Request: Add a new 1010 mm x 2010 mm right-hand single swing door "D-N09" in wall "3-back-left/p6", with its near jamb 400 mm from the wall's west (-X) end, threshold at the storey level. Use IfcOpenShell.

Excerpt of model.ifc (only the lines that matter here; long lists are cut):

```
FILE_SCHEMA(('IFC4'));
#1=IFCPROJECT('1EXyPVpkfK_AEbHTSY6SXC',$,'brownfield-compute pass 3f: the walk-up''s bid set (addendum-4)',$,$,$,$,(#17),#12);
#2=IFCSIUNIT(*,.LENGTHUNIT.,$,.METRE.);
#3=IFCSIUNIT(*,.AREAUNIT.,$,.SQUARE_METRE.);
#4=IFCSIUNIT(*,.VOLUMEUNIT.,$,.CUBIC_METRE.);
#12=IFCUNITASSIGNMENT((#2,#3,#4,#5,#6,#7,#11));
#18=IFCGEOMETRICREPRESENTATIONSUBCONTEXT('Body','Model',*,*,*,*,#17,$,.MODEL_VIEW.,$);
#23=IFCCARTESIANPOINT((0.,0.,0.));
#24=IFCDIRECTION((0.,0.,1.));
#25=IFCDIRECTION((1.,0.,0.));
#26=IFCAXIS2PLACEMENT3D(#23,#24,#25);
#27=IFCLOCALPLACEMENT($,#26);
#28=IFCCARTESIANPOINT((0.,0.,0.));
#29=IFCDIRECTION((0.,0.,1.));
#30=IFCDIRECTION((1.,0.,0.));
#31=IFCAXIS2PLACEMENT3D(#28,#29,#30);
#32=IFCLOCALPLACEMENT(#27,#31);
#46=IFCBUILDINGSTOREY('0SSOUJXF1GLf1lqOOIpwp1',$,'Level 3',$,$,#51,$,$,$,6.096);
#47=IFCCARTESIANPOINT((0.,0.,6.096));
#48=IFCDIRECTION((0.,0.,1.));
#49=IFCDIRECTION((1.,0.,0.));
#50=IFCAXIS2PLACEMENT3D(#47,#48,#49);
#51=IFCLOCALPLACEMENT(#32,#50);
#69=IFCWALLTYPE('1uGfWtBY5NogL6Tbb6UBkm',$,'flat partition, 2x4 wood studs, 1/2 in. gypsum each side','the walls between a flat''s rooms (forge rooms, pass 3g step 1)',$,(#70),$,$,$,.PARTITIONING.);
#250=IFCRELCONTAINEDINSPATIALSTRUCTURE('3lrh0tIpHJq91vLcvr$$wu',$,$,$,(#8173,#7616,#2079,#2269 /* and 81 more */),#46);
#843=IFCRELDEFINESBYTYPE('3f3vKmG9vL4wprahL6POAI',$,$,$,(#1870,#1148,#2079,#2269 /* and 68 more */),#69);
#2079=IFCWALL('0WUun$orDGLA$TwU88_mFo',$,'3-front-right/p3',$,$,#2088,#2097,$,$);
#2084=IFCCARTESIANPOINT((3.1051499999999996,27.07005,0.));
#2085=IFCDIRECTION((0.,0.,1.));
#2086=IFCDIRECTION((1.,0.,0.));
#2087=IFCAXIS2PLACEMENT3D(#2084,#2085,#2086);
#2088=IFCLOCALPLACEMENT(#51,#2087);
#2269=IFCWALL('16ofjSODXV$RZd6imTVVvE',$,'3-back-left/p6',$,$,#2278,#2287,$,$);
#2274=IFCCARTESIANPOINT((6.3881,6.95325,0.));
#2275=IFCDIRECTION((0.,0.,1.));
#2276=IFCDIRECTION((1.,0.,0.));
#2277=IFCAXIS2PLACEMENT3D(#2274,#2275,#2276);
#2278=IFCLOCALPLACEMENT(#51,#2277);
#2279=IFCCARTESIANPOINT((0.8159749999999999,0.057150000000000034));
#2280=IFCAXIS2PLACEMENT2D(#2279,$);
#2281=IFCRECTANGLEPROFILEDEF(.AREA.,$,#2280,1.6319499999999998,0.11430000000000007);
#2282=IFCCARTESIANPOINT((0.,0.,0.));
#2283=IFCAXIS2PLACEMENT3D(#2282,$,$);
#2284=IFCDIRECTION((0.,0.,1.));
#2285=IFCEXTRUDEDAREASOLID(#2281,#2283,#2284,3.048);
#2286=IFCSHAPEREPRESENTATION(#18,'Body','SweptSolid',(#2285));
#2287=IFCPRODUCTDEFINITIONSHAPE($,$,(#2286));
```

```python
import numpy as np
import ifcopenshell
import ifcopenshell.api.feature
import ifcopenshell.api.geometry
import ifcopenshell.api.root
import ifcopenshell.api.spatial
import ifcopenshell.geom
import ifcopenshell.util.element
import ifcopenshell.util.placement
import ifcopenshell.util.representation
import ifcopenshell.util.shape
import ifcopenshell.util.unit

model = ifcopenshell.open("model.ifc")
unit_scale = ifcopenshell.util.unit.calculate_unit_scale(model)
settings = ifcopenshell.geom.settings()


def volume(element):
    """Net volume in cubic metres, openings subtracted."""
    shape = ifcopenshell.geom.create_shape(settings, element)
    return ifcopenshell.util.shape.get_volume(shape.geometry)


wall = model.by_id(2269)
storey = ifcopenshell.util.element.get_container(wall, ifc_class="IfcBuildingStorey")
context = ifcopenshell.util.representation.get_context(model, "Model", "Body", "MODEL_VIEW")
before = volume(wall)

width, height, from_end, sill = 1.01, 2.01, 0.4, 0.0  # metres

# The wall runs along its own X axis, and the end named is its -X end.
wall_shape = ifcopenshell.geom.create_shape(settings, wall)
x, y, z = ifcopenshell.util.shape.get_vertices(wall_shape.geometry).T
start = x.min() + from_end
face, thickness = float(y.min()), float(y.max() - y.min())
wall_matrix = ifcopenshell.util.placement.get_local_placement(wall.ObjectPlacement)
level = ifcopenshell.util.placement.get_local_placement(storey.ObjectPlacement)[2, 3]


def in_wall(x, y):
    """Placement at x, y metres in the wall's axes, at sill height."""
    matrix = wall_matrix.copy()
    matrix[:, 3] = wall_matrix @ np.array([x / unit_scale, y / unit_scale, 0.0, 1.0])
    matrix[2, 3] = level + sill / unit_scale
    return matrix


# Opening: a box that overshoots both wall faces by 50 mm.
opening = ifcopenshell.api.root.create_entity(model, ifc_class="IfcOpeningElement", predefined_type="OPENING")
box = ifcopenshell.api.geometry.add_wall_representation(
    model, context=context, length=width, height=height, thickness=thickness + 0.1
)
ifcopenshell.api.geometry.assign_representation(model, product=opening, representation=box)
ifcopenshell.api.geometry.edit_object_placement(model, product=opening, matrix=in_wall(start, face - 0.05), is_si=False)
ifcopenshell.api.feature.add_feature(model, feature=opening, element=wall)

door = ifcopenshell.api.root.create_entity(model, ifc_class="IfcDoor", name="D-N09", predefined_type="DOOR")
door.OverallWidth, door.OverallHeight = width / unit_scale, height / unit_scale
door.OperationType = "SINGLE_SWING_RIGHT"
body = ifcopenshell.api.geometry.add_door_representation(
    model,
    context=context,
    overall_width=door.OverallWidth,
    overall_height=door.OverallHeight,
    operation_type="SINGLE_SWING_RIGHT",
    lining_properties={"LiningDepth": thickness / unit_scale, "ThresholdDepth": thickness / unit_scale},
)
ifcopenshell.api.geometry.assign_representation(model, product=door, representation=body)
ifcopenshell.api.spatial.assign_container(model, products=[door], relating_structure=storey)
ifcopenshell.api.feature.add_filling(model, opening=opening, element=door)

# The lining spans the wall, so the door starts at the wall face.
ifcopenshell.api.geometry.edit_object_placement(model, product=door, matrix=in_wall(start, face), is_si=False)

after = volume(wall)

print(f"wall volume {before:.3f} -> {after:.3f} m3")

model.write("model_rev.ifc")
```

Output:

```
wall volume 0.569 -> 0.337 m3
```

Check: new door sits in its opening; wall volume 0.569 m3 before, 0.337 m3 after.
